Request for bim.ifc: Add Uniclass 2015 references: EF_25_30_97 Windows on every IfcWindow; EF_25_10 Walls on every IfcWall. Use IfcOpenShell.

First a look at what the model holds.

```python
import ifcopenshell

model = ifcopenshell.open("bim.ifc")
print(model.schema)
print("classifications:", [c.Name for c in model.by_type("IfcClassification")])
for ifc_class in ("IfcDoor", "IfcRoof", "IfcStair", "IfcWall", "IfcWindow"):
    print(ifc_class, len(model.by_type(ifc_class)))
```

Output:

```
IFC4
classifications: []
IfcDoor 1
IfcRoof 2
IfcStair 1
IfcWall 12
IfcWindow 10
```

```python
import ifcopenshell
import ifcopenshell.api.classification

model = ifcopenshell.open("bim.ifc")

system = ifcopenshell.api.classification.add_classification(model, classification="Uniclass 2015")

codes = {
    "IfcWindow": ("EF_25_30_97", "Windows"),
    "IfcWall": ("EF_25_10", "Walls"),
}
for ifc_class, (code, name) in codes.items():
    products = model.by_type(ifc_class)
    ifcopenshell.api.classification.add_reference(
        model, products=products, classification=system, identification=code, name=name
    )
    print(code, len(products))

model.write("bim_rev.ifc")
```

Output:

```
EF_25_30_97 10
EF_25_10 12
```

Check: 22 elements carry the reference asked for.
